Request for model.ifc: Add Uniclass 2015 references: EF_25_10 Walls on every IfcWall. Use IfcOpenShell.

First a look at what the model holds.

```python
import ifcopenshell

model = ifcopenshell.open("model.ifc")
print(model.schema)
print("classifications:", [c.Name for c in model.by_type("IfcClassification")])
for ifc_class in ("IfcDoor", "IfcRoof", "IfcStair", "IfcWall", "IfcWindow"):
    print(ifc_class, len(model.by_type(ifc_class)))
```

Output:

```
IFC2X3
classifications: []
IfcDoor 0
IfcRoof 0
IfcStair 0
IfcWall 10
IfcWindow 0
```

```python
import ifcopenshell
import ifcopenshell.api.classification

model = ifcopenshell.open("model.ifc")

# IFC2X3 requires Source and Edition and has no link from the project to the system.
system = model.create_entity("IfcClassification", Source="NBS", Edition="2015", Name="Uniclass 2015")

codes = {
    "IfcWall": ("EF_25_10", "Walls"),
}
for ifc_class, (code, name) in codes.items():
    products = model.by_type(ifc_class)
    ifcopenshell.api.classification.add_reference(
        model, products=products, classification=system, identification=code, name=name
    )
    print(code, len(products))

model.write("model_rev.ifc")
```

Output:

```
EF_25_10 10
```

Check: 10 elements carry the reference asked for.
